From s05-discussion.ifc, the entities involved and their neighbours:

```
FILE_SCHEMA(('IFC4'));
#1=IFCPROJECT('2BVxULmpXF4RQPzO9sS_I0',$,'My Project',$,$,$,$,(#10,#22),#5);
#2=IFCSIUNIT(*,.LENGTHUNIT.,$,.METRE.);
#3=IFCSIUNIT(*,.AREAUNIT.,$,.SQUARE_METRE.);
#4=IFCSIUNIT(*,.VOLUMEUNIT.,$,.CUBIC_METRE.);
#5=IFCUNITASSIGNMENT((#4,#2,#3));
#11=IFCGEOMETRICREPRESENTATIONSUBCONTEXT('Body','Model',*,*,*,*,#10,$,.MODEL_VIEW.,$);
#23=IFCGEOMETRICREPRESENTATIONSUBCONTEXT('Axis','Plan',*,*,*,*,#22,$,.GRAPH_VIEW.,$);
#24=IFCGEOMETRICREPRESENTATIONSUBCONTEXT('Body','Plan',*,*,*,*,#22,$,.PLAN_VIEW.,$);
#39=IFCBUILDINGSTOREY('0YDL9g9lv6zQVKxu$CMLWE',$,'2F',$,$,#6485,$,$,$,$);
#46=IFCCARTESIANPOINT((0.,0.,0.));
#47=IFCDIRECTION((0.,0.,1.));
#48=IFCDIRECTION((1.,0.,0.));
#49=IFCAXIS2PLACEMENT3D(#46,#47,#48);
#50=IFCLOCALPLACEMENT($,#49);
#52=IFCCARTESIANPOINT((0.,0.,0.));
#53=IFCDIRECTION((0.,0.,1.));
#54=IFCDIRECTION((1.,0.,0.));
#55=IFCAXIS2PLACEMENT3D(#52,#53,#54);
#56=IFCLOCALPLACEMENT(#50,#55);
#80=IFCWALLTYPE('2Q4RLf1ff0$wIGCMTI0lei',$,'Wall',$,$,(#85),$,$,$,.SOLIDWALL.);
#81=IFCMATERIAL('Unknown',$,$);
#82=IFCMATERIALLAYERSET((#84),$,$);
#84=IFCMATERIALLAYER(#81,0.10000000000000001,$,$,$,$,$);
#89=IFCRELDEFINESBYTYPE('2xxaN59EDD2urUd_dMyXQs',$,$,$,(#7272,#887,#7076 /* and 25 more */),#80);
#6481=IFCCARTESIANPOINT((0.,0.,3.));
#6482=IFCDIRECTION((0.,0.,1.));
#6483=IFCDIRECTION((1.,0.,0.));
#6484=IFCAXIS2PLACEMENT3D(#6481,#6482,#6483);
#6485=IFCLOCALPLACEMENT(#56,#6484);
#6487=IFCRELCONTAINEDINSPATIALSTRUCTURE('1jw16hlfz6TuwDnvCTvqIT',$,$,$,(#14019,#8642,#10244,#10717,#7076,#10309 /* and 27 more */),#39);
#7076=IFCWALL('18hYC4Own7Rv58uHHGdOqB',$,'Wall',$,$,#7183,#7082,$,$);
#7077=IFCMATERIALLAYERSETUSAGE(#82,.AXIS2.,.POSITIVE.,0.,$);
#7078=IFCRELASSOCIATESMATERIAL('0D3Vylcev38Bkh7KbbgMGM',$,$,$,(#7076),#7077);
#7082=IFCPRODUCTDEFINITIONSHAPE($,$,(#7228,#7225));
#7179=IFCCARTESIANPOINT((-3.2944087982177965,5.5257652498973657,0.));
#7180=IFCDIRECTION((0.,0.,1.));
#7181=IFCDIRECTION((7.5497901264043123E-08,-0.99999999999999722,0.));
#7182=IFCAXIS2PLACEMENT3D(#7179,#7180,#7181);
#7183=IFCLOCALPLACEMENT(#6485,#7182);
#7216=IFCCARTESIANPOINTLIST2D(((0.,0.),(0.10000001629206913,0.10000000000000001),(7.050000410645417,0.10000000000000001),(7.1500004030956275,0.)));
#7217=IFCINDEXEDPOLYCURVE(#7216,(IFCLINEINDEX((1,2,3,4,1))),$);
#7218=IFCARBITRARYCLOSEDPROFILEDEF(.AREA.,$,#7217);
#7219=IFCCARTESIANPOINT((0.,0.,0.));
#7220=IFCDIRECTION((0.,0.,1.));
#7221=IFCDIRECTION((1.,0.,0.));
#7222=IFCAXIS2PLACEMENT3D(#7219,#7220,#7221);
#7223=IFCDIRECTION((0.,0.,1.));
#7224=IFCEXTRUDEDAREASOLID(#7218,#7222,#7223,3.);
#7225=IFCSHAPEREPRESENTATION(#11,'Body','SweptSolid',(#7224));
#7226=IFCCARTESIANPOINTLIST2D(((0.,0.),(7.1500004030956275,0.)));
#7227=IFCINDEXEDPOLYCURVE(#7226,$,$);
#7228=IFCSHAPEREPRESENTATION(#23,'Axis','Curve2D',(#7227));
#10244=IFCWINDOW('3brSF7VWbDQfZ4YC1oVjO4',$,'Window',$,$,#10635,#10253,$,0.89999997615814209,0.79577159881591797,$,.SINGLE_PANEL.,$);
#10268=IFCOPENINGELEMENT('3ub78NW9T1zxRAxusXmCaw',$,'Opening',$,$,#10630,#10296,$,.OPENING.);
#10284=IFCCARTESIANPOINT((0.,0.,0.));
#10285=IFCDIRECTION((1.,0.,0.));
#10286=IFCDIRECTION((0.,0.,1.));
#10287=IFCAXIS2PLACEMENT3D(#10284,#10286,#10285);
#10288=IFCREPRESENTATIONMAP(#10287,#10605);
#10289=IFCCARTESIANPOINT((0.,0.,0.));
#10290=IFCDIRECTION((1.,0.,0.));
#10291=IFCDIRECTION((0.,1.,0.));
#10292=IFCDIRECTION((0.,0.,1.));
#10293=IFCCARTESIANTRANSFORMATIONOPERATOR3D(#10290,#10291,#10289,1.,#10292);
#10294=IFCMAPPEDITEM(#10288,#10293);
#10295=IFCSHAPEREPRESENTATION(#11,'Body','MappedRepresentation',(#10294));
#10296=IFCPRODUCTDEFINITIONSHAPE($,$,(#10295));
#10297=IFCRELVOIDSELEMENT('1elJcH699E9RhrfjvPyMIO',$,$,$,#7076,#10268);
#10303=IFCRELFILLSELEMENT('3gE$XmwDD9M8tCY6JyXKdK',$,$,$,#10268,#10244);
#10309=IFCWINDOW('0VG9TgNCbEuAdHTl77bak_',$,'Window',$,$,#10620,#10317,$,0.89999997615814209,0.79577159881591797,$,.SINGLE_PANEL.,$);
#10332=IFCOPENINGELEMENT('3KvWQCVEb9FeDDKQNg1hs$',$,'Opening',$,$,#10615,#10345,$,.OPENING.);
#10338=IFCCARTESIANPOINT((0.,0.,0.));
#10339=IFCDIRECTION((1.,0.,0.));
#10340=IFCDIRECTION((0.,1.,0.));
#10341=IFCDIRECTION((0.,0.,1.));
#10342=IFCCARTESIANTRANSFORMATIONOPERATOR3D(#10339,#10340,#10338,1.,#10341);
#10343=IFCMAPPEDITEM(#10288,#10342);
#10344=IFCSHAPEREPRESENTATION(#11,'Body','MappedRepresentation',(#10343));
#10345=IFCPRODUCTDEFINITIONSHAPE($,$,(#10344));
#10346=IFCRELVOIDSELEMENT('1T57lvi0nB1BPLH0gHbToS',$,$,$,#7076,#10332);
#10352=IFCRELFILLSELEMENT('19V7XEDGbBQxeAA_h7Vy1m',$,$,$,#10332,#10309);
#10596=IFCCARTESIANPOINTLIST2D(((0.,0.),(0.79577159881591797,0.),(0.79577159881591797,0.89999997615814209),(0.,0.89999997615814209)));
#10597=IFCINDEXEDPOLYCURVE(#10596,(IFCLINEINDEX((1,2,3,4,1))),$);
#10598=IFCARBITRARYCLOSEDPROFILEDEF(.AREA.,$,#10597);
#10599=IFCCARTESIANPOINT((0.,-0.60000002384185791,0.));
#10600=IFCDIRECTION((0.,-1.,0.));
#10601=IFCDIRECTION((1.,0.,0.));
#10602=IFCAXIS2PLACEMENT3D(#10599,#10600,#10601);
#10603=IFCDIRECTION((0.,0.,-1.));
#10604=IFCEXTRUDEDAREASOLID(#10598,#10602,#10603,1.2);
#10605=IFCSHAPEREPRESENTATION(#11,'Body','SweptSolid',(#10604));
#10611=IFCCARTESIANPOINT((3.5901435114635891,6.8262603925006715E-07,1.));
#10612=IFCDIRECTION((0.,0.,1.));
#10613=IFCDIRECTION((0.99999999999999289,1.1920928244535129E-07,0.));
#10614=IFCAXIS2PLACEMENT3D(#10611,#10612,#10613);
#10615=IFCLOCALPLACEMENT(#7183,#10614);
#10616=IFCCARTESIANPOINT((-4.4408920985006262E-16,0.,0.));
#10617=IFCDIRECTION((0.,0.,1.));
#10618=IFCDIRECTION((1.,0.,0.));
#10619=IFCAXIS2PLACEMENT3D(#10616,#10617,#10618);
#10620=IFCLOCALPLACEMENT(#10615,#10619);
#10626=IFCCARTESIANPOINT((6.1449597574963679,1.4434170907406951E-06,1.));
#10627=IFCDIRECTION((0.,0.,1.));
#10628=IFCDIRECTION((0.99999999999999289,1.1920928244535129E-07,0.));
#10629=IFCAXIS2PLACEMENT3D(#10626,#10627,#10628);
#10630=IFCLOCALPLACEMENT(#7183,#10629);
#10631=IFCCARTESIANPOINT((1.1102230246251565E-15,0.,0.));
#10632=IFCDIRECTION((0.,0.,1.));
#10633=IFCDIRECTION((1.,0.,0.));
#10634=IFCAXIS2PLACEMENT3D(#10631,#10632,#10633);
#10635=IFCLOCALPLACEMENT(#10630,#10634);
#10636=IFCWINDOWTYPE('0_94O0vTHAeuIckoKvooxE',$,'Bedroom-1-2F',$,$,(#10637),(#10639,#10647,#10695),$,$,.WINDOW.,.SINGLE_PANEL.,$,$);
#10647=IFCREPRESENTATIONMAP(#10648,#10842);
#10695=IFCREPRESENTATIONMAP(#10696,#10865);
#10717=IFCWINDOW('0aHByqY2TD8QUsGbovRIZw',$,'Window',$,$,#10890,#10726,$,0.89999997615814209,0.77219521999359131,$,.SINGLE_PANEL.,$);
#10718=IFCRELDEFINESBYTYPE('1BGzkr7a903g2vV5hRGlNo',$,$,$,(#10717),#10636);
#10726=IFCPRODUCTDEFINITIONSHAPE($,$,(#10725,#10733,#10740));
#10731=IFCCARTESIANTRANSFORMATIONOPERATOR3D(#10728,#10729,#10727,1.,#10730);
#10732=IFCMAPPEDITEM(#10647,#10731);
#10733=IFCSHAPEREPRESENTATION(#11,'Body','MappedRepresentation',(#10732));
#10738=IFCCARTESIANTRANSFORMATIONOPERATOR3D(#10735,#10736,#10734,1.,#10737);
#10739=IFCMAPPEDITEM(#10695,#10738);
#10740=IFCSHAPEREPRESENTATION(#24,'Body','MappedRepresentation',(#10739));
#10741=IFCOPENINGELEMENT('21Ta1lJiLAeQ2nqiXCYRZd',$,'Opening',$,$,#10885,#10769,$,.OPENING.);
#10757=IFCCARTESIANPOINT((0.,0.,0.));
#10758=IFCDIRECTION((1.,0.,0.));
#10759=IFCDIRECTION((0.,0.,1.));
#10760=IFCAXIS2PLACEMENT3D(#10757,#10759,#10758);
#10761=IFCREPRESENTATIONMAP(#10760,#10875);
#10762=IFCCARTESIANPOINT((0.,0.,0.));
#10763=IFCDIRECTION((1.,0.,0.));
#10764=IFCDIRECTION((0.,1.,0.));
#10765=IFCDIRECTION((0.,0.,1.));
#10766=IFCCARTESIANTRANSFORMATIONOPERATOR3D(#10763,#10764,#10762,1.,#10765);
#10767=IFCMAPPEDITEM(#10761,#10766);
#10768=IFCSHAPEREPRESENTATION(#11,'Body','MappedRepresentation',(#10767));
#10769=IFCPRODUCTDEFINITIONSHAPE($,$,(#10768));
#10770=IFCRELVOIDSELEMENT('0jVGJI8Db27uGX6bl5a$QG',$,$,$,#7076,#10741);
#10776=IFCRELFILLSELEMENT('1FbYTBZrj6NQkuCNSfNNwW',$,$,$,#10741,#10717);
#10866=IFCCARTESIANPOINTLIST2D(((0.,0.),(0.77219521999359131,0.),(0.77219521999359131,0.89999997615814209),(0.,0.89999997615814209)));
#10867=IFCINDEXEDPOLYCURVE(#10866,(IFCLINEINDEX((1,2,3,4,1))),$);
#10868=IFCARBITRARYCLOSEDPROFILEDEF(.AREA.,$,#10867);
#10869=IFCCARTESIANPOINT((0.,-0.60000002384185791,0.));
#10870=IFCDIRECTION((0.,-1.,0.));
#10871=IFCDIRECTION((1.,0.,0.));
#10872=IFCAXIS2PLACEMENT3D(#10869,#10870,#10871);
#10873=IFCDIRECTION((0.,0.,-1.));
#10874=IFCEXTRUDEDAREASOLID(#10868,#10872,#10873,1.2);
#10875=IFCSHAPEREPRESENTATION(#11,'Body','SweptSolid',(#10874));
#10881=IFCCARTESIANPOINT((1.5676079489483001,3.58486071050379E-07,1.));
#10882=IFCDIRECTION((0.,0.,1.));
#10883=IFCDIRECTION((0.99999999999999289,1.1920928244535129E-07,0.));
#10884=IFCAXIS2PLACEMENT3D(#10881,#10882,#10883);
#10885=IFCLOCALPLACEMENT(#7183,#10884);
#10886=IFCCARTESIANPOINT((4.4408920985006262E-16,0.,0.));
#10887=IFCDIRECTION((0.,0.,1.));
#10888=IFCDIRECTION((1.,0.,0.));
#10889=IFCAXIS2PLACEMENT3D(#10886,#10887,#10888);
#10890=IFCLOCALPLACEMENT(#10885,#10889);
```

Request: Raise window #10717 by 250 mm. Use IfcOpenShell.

```python
import numpy as np
import ifcopenshell
import ifcopenshell.api.geometry
import ifcopenshell.util.placement
import ifcopenshell.util.unit

model = ifcopenshell.open("s05-discussion.ifc")
unit_scale = ifcopenshell.util.unit.calculate_unit_scale(model)

window = model.by_guid("0aHByqY2TD8QUsGbovRIZw")
opening = window.FillsVoids[0].RelatingOpeningElement
dz = 0.25 / unit_scale

shift = np.array([0.0, 0.0, dz])
# The window is placed relative to its opening, so it follows when the opening moves.
matrix = ifcopenshell.util.placement.get_local_placement(opening.ObjectPlacement)
matrix[:3, 3] += shift
ifcopenshell.api.geometry.edit_object_placement(
    model, product=opening, matrix=matrix, is_si=False, should_transform_children=True
)

print(f"moved by {dz * unit_scale:+.3f} m")

model.write("s05-discussion_edited.ifc")
```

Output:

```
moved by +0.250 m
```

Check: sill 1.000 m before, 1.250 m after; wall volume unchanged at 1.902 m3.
